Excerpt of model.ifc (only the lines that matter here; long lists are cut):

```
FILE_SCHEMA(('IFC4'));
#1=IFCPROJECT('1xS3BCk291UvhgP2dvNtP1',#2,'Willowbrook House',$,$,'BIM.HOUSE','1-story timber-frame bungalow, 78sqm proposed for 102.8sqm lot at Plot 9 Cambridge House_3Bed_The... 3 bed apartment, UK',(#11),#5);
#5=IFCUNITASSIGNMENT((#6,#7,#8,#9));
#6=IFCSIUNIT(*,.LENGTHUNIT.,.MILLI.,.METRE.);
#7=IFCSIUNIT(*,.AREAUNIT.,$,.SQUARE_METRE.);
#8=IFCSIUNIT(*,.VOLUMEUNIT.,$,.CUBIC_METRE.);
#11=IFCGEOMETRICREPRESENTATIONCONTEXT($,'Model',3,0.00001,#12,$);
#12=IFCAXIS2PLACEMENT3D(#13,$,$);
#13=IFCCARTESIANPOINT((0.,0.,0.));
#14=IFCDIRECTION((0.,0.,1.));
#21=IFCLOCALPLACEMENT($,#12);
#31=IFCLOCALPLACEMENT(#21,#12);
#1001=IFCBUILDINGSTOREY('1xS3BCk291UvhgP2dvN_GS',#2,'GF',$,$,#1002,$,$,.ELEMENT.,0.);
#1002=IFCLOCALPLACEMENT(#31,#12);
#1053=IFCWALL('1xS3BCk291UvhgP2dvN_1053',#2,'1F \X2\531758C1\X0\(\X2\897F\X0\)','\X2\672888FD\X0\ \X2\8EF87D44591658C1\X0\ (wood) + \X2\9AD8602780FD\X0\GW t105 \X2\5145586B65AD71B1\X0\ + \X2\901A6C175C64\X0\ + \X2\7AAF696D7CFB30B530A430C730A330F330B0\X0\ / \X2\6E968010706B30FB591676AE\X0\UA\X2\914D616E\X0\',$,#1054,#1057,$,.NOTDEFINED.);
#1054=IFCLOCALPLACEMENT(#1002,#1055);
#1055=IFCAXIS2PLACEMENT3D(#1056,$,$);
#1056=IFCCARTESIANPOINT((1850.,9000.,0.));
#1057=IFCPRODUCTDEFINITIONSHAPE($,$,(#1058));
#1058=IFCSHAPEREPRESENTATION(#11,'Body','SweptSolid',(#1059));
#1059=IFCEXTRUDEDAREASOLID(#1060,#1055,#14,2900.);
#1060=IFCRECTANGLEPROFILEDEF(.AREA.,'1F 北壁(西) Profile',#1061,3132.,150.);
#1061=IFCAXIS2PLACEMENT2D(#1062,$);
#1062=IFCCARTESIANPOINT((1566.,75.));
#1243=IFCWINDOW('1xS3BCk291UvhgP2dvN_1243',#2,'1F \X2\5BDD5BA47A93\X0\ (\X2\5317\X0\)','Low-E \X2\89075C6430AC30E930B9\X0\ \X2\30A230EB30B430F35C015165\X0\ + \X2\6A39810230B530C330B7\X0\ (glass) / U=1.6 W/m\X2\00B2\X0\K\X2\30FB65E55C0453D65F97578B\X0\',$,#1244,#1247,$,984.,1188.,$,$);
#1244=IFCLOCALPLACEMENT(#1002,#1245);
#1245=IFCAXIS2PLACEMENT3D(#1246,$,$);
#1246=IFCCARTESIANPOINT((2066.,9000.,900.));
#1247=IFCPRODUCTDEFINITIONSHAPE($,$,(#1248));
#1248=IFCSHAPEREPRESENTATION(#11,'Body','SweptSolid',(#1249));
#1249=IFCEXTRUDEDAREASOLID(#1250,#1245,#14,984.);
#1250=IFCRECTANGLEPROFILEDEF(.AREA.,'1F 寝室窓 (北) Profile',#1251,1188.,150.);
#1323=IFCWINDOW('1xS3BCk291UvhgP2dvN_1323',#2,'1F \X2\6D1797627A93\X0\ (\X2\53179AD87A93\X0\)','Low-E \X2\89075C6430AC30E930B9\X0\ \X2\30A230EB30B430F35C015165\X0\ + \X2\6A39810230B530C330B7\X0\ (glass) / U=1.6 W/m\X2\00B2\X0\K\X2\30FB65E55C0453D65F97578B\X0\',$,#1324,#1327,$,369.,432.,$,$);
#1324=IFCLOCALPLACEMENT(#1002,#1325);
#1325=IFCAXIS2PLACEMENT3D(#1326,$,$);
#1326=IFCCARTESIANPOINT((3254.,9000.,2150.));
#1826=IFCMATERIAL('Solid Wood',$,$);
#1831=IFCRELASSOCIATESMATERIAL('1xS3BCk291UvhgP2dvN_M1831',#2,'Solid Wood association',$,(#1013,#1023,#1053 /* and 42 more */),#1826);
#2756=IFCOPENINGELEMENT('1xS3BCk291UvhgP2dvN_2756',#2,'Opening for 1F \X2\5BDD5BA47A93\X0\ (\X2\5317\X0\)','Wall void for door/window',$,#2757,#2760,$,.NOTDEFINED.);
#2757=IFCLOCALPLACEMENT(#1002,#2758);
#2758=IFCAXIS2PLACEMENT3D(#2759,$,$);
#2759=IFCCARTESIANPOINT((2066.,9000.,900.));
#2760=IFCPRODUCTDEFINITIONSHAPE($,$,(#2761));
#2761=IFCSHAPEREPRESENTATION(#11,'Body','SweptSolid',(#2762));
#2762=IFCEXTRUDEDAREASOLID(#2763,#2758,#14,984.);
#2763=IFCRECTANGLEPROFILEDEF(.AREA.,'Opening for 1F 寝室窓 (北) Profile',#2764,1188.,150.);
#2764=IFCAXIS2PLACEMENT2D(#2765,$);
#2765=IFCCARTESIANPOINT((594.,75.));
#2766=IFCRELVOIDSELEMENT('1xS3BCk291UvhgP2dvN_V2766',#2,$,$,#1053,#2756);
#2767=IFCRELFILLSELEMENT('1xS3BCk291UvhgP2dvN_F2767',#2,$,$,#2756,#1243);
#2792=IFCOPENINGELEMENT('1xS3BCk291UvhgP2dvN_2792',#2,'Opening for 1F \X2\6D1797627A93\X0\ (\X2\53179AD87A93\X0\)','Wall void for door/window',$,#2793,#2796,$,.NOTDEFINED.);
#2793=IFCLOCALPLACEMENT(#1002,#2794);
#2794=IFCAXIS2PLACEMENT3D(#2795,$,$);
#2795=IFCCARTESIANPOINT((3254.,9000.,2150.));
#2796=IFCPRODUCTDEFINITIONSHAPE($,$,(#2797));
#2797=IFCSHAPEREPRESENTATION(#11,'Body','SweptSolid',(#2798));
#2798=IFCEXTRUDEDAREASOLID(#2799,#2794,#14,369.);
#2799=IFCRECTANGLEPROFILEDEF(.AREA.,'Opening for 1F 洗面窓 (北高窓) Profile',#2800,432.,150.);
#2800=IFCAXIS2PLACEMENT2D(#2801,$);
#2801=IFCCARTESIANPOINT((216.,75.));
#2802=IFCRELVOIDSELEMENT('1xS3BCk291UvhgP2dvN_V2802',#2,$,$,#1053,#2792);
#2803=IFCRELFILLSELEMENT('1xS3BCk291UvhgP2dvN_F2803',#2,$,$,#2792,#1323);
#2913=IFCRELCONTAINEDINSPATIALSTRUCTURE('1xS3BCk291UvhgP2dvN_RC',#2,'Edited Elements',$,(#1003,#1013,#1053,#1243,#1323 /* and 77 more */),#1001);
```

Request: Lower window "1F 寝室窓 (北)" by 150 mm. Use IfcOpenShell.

```python
import numpy as np
import ifcopenshell
import ifcopenshell.api.geometry
import ifcopenshell.util.placement
import ifcopenshell.util.unit

model = ifcopenshell.open("model.ifc")
unit_scale = ifcopenshell.util.unit.calculate_unit_scale(model)

window = model.by_guid("1xS3BCk291UvhgP2dvN_1243")
opening = window.FillsVoids[0].RelatingOpeningElement
dz = -0.15 / unit_scale

shift = np.array([0.0, 0.0, dz])
# The window is not placed relative to its opening, so move both.
for product in (opening, window):
    matrix = ifcopenshell.util.placement.get_local_placement(product.ObjectPlacement)
    matrix[:3, 3] += shift
    ifcopenshell.api.geometry.edit_object_placement(model, product=product, matrix=matrix, is_si=False)

print(f"moved by {dz * unit_scale:+.3f} m")

model.write("model_v2.ifc")
```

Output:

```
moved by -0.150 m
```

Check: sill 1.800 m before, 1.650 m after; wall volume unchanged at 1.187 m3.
